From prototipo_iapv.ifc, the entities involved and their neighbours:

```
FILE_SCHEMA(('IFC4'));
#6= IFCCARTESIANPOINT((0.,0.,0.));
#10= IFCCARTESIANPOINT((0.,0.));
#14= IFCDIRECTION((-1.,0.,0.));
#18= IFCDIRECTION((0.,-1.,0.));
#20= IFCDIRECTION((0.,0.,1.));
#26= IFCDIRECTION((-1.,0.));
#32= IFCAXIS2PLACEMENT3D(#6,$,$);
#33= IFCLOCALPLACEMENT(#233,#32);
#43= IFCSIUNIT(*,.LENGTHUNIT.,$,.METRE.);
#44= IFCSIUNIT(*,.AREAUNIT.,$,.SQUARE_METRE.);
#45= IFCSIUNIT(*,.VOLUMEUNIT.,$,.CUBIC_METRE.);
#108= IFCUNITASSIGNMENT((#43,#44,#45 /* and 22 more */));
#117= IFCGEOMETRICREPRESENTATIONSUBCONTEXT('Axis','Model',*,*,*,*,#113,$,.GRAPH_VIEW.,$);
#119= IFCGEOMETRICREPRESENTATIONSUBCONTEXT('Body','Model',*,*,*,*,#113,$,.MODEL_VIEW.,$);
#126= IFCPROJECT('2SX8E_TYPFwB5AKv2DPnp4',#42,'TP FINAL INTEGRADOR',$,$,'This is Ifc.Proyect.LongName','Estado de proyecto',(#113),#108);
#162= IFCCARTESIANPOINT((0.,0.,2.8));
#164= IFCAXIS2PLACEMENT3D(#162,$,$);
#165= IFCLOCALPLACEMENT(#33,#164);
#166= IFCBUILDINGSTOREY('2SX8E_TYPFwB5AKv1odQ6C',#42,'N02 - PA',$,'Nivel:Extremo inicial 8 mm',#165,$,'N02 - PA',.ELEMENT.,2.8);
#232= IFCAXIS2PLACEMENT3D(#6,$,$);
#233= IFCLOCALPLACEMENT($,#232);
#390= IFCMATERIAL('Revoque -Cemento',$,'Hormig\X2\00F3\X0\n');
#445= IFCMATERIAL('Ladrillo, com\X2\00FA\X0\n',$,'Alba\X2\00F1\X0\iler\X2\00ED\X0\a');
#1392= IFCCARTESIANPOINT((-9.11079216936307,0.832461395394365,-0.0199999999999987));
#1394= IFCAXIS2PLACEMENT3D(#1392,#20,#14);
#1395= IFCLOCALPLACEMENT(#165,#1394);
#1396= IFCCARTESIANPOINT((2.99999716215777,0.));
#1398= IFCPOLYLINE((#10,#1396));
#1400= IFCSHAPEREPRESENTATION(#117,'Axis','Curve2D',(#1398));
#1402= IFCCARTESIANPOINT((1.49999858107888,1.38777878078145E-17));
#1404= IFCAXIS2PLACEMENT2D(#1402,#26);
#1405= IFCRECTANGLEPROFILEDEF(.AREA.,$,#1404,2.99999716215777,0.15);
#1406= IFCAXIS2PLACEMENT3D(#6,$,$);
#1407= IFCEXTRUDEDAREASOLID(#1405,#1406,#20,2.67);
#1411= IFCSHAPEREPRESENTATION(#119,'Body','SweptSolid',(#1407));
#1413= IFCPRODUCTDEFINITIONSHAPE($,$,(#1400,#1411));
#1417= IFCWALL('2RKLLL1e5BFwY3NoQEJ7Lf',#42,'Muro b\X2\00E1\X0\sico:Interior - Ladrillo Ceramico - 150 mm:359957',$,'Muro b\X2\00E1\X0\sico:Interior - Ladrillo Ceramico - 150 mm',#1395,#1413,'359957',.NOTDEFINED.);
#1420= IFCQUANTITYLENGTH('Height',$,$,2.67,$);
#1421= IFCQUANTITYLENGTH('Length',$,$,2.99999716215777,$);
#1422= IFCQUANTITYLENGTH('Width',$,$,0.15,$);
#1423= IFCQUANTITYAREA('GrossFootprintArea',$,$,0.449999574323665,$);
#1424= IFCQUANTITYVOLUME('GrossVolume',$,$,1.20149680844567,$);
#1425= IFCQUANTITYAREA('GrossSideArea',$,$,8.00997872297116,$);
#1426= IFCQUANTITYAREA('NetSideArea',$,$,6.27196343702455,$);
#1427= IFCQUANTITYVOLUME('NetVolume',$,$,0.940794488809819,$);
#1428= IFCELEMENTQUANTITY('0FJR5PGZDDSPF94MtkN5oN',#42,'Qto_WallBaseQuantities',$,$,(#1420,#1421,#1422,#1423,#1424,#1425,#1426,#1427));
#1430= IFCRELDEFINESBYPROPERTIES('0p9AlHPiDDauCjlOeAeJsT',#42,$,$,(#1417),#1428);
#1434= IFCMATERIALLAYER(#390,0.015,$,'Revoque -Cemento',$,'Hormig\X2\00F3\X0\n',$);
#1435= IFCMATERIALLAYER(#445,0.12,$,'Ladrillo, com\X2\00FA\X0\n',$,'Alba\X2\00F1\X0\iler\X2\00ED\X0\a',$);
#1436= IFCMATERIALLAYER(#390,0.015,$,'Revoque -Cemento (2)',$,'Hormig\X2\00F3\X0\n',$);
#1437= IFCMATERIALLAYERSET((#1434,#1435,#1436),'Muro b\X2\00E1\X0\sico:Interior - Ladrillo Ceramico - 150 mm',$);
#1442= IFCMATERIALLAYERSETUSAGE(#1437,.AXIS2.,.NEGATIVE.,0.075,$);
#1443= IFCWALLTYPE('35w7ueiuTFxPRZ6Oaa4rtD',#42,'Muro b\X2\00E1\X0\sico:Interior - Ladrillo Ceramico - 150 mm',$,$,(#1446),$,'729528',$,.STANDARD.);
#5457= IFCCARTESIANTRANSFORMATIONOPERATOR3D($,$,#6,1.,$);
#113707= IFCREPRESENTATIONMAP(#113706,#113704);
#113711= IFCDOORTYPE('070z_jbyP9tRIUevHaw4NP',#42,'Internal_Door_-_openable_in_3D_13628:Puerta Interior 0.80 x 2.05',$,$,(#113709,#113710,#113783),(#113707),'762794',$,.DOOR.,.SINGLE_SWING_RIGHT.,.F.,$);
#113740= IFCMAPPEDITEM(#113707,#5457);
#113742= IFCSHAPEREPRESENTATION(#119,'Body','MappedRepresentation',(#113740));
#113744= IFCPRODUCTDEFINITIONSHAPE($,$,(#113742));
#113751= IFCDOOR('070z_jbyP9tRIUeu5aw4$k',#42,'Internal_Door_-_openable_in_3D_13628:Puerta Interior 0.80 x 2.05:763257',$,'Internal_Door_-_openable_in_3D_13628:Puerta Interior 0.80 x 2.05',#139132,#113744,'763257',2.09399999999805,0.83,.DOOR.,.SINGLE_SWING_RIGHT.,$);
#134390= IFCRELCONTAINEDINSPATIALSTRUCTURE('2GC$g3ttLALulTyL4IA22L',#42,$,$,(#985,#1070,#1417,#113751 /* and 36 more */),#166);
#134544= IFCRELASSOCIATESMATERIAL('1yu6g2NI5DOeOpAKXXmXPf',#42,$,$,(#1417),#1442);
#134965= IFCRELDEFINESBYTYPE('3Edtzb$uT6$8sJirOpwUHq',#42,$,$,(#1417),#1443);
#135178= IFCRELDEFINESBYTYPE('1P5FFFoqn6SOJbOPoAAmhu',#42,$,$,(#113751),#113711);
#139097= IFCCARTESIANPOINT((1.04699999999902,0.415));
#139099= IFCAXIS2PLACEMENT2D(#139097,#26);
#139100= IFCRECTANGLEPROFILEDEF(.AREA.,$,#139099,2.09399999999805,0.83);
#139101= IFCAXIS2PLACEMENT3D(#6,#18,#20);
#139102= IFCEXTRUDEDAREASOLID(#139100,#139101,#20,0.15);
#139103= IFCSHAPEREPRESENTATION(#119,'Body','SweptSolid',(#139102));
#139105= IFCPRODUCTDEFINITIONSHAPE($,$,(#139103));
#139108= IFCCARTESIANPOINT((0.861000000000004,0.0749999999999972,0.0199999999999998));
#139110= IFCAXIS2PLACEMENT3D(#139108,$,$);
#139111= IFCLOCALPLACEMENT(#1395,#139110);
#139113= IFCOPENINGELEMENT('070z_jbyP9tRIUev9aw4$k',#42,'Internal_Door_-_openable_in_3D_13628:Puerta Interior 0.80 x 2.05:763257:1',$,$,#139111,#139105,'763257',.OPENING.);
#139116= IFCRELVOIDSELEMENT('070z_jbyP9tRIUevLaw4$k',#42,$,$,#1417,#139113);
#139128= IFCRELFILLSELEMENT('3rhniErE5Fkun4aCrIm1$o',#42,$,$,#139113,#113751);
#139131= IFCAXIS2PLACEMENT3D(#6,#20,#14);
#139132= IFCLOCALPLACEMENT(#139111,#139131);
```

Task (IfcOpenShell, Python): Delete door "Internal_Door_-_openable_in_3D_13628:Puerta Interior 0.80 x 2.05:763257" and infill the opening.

```python
import ifcopenshell
import ifcopenshell.api.feature
import ifcopenshell.api.pset
import ifcopenshell.api.root
import ifcopenshell.geom
import ifcopenshell.util.element
import ifcopenshell.util.shape
import ifcopenshell.util.unit

model = ifcopenshell.open("prototipo_iapv.ifc")
area_scale = ifcopenshell.util.unit.calculate_unit_scale(model, "AREAUNIT")
volume_scale = ifcopenshell.util.unit.calculate_unit_scale(model, "VOLUMEUNIT")
settings = ifcopenshell.geom.settings()


def volume(element):
    """Net volume in cubic metres, openings subtracted."""
    shape = ifcopenshell.geom.create_shape(settings, element)
    return ifcopenshell.util.shape.get_volume(shape.geometry)


door = model.by_id(113751)
opening = door.FillsVoids[0].RelatingOpeningElement
wall = opening.VoidsElements[0].RelatingBuildingElement
before = volume(wall)

ifcopenshell.api.root.remove_product(model, product=door)
ifcopenshell.api.feature.remove_feature(model, feature=opening)

after = volume(wall)
thickness = 0.15  # wall thickness in metres

# Update the wall's stored quantities.
qto = model.by_id(ifcopenshell.util.element.get_pset(wall, "Qto_WallBaseQuantities", should_inherit=False)["id"])
ifcopenshell.api.pset.edit_qto(model, qto=qto, properties={
    "NetSideArea": after / thickness / area_scale,
    "NetVolume": after / volume_scale,
})

print(f"wall volume {before:.3f} -> {after:.3f} m3")

model.write("prototipo_iapv-out.ifc")
```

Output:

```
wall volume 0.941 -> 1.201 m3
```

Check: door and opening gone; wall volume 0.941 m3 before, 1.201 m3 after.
